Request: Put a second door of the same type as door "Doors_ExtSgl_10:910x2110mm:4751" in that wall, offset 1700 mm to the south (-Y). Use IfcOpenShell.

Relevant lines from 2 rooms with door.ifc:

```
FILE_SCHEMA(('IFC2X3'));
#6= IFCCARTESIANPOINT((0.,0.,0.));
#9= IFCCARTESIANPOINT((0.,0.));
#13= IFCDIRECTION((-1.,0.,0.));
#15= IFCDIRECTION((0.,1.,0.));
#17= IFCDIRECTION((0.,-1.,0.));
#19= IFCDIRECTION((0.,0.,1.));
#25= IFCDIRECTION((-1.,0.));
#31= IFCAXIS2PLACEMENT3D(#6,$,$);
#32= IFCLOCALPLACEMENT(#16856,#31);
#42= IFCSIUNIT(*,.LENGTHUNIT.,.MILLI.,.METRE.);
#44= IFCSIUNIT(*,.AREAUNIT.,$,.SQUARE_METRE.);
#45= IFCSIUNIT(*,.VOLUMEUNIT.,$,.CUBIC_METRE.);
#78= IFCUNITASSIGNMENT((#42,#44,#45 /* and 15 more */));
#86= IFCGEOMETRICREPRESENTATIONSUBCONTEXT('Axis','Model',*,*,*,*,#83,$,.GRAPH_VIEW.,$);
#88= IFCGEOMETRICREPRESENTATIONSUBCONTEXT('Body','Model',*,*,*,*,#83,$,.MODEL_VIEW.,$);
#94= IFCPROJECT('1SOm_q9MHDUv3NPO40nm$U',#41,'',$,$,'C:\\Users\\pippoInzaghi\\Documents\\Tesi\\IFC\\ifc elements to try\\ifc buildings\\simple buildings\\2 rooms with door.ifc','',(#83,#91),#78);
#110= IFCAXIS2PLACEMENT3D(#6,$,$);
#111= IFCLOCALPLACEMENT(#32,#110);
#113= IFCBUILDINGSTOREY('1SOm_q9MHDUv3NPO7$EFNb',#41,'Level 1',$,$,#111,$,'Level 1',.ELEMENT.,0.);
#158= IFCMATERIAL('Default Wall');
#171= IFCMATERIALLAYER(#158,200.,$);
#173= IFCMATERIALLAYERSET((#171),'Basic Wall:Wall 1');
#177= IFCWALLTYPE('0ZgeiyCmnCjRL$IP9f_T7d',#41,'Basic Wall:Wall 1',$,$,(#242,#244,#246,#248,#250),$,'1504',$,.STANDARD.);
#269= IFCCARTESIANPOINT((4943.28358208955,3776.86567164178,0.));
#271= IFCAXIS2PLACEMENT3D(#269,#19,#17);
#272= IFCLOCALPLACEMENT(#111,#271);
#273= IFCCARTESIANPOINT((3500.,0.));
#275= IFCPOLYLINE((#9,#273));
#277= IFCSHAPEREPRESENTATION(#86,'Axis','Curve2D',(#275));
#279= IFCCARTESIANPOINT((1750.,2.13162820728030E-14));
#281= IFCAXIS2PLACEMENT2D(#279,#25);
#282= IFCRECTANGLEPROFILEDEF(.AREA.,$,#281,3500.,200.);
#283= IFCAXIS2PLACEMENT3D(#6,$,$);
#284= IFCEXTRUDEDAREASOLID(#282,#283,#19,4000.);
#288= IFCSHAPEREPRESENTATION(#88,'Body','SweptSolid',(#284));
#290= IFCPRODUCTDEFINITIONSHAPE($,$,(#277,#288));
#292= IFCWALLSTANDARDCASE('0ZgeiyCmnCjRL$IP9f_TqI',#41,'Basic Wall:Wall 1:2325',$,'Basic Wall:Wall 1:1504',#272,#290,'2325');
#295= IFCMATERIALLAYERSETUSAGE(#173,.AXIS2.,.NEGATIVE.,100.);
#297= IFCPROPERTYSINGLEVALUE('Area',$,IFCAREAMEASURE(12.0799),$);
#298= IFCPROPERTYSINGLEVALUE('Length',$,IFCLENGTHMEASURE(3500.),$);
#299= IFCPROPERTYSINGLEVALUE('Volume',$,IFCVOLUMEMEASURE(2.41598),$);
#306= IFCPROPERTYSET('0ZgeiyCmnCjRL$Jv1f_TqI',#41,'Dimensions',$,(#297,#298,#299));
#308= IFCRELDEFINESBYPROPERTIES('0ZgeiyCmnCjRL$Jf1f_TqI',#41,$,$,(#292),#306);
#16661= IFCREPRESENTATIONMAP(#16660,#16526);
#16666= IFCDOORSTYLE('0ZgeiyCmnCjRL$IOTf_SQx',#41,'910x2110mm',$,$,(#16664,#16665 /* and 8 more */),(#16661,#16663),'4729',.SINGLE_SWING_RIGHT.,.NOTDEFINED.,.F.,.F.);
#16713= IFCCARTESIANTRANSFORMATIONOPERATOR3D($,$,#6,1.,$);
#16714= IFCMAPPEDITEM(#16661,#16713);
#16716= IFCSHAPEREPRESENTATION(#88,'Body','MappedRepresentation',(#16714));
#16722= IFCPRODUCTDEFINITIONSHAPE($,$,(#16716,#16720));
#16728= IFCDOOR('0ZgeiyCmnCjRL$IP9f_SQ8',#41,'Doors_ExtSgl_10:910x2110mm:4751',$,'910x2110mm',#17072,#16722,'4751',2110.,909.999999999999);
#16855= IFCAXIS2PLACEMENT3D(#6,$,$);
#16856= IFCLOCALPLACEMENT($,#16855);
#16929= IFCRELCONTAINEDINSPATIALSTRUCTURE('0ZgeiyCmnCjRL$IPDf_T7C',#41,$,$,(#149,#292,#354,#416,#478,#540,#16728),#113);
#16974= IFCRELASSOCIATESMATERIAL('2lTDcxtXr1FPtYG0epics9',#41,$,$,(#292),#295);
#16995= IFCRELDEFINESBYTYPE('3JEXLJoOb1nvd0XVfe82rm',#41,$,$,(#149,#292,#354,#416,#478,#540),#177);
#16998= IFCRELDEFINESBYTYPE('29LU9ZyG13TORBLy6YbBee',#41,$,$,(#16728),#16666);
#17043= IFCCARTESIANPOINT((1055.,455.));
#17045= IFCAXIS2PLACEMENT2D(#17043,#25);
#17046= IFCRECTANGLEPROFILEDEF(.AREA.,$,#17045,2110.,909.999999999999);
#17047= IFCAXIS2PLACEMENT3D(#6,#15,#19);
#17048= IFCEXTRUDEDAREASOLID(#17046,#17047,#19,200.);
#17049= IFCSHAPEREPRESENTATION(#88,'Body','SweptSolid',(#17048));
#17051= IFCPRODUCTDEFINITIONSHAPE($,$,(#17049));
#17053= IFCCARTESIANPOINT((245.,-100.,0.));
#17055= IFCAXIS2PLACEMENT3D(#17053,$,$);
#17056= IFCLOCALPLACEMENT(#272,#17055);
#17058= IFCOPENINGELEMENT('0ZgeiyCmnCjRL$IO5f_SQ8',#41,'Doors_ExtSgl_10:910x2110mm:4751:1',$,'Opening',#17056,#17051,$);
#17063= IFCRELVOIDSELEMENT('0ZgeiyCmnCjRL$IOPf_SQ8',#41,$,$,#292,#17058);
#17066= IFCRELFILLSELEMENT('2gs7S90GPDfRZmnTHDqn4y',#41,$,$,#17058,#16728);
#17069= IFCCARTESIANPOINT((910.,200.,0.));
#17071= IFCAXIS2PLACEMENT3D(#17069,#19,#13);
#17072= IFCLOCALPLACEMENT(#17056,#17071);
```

```python
import ifcopenshell
import ifcopenshell.api.feature
import ifcopenshell.api.geometry
import ifcopenshell.api.pset
import ifcopenshell.api.root
import ifcopenshell.geom
import ifcopenshell.util.element
import ifcopenshell.util.placement
import ifcopenshell.util.shape
import ifcopenshell.util.unit

model = ifcopenshell.open("2 rooms with door.ifc")
unit_scale = ifcopenshell.util.unit.calculate_unit_scale(model)
area_scale = ifcopenshell.util.unit.calculate_unit_scale(model, "AREAUNIT")
volume_scale = ifcopenshell.util.unit.calculate_unit_scale(model, "VOLUMEUNIT")
settings = ifcopenshell.geom.settings()


def volume(element):
    """Net volume in cubic metres, openings subtracted."""
    shape = ifcopenshell.geom.create_shape(settings, element)
    return ifcopenshell.util.shape.get_volume(shape.geometry)


def reuse_history(source, copy):
    """copy_class also copies each property set's owner history, people and application; keep the originals."""
    for rel in copy.IsDefinedBy:
        if rel.is_a("IfcRelDefinesByProperties") and (history := rel.RelatingPropertyDefinition.OwnerHistory):
            rel.RelatingPropertyDefinition.OwnerHistory = source.OwnerHistory
            ifcopenshell.util.element.remove_deep2(model, history)


door = model.by_id(16728)
opening = door.FillsVoids[0].RelatingOpeningElement
wall = opening.VoidsElements[0].RelatingBuildingElement
before = volume(wall)
shift = ifcopenshell.util.placement.get_local_placement(wall.ObjectPlacement)[:3, 0] * 1.7 / unit_scale

# copy_class copies the void relationship, type, container and properties, but no geometry.
new_opening = ifcopenshell.api.root.copy_class(model, product=opening)
new_opening.Representation = ifcopenshell.util.element.copy_deep(
    model, opening.Representation, exclude=["IfcGeometricRepresentationContext", "IfcRepresentationMap"]
)
new_opening.Name = "Doors_ExtSgl_10:910x2110mm"
new_door = ifcopenshell.api.root.copy_class(model, product=door)
new_door.Representation = ifcopenshell.util.element.copy_deep(
    model, door.Representation, exclude=["IfcGeometricRepresentationContext", "IfcRepresentationMap"]
)
new_door.Name = "Doors_ExtSgl_10:910x2110mm"
new_door.Tag = None
reuse_history(door, new_door)
fills = ifcopenshell.api.feature.add_filling(model, opening=new_opening, element=new_door)
fills.OwnerHistory = new_door.OwnerHistory  # required in IFC2X3

for old, new in ((opening, new_opening), (door, new_door)):
    matrix = ifcopenshell.util.placement.get_local_placement(old.ObjectPlacement)
    matrix[:3, 3] += shift
    ifcopenshell.api.geometry.edit_object_placement(model, product=new, matrix=matrix, is_si=False)

after = volume(wall)
thickness = 0.2  # wall thickness in metres

# Update the wall's stored quantities.
pset = model.by_id(ifcopenshell.util.element.get_pset(wall, "Dimensions", should_inherit=False)["id"])
ifcopenshell.api.pset.edit_pset(model, pset=pset, properties={
    "Area": model.create_entity("IfcAreaMeasure", after / thickness / area_scale),
    "Volume": model.create_entity("IfcVolumeMeasure", after / volume_scale),
})

print(f"wall volume {before:.3f} -> {after:.3f} m3")

model.write("2 rooms with door_rev.ifc")
```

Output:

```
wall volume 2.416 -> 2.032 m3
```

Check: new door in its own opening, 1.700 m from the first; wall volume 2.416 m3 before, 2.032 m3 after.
